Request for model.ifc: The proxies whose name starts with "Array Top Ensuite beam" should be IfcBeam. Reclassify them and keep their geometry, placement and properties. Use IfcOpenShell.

First a look at what the model holds.

```python
import re

import ifcopenshell

model = ifcopenshell.open("model.ifc")
print(model.schema)
seen = {}
for e in model.by_type("IfcBuildingElementProxy"):
    name = re.sub(r":\d+(:\d+)?$", "", e.Name or "")  # drop the element id that some exporters append
    seen[name] = seen.get(name, 0) + 1
for name, count in sorted(seen.items()):
    print(count, "x", name)
```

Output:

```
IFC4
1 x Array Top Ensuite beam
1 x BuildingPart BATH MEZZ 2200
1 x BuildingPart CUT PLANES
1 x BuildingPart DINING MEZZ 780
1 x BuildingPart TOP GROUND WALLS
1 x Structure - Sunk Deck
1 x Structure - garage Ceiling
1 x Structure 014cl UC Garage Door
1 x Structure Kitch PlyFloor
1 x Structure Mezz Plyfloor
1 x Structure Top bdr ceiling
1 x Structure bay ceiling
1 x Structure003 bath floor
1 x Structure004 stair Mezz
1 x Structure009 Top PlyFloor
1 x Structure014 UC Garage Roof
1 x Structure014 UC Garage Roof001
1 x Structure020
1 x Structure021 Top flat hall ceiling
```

```python
import ifcopenshell
import ifcopenshell.api.root

model = ifcopenshell.open("model.ifc")

proxies = [e.id() for e in model.by_type("IfcBuildingElementProxy") if (e.Name or "").startswith("Array Top Ensuite beam")]
for step_id in proxies:
    proxy = model.by_id(step_id)
    ifcopenshell.api.root.reassign_class(model, product=proxy, ifc_class="IfcBeam")

print(sum(model.by_id(i).is_a("IfcBeam") for i in proxies), "reclassified")

model.write("model_edited.ifc")
```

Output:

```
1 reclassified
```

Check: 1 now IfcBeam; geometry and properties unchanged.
